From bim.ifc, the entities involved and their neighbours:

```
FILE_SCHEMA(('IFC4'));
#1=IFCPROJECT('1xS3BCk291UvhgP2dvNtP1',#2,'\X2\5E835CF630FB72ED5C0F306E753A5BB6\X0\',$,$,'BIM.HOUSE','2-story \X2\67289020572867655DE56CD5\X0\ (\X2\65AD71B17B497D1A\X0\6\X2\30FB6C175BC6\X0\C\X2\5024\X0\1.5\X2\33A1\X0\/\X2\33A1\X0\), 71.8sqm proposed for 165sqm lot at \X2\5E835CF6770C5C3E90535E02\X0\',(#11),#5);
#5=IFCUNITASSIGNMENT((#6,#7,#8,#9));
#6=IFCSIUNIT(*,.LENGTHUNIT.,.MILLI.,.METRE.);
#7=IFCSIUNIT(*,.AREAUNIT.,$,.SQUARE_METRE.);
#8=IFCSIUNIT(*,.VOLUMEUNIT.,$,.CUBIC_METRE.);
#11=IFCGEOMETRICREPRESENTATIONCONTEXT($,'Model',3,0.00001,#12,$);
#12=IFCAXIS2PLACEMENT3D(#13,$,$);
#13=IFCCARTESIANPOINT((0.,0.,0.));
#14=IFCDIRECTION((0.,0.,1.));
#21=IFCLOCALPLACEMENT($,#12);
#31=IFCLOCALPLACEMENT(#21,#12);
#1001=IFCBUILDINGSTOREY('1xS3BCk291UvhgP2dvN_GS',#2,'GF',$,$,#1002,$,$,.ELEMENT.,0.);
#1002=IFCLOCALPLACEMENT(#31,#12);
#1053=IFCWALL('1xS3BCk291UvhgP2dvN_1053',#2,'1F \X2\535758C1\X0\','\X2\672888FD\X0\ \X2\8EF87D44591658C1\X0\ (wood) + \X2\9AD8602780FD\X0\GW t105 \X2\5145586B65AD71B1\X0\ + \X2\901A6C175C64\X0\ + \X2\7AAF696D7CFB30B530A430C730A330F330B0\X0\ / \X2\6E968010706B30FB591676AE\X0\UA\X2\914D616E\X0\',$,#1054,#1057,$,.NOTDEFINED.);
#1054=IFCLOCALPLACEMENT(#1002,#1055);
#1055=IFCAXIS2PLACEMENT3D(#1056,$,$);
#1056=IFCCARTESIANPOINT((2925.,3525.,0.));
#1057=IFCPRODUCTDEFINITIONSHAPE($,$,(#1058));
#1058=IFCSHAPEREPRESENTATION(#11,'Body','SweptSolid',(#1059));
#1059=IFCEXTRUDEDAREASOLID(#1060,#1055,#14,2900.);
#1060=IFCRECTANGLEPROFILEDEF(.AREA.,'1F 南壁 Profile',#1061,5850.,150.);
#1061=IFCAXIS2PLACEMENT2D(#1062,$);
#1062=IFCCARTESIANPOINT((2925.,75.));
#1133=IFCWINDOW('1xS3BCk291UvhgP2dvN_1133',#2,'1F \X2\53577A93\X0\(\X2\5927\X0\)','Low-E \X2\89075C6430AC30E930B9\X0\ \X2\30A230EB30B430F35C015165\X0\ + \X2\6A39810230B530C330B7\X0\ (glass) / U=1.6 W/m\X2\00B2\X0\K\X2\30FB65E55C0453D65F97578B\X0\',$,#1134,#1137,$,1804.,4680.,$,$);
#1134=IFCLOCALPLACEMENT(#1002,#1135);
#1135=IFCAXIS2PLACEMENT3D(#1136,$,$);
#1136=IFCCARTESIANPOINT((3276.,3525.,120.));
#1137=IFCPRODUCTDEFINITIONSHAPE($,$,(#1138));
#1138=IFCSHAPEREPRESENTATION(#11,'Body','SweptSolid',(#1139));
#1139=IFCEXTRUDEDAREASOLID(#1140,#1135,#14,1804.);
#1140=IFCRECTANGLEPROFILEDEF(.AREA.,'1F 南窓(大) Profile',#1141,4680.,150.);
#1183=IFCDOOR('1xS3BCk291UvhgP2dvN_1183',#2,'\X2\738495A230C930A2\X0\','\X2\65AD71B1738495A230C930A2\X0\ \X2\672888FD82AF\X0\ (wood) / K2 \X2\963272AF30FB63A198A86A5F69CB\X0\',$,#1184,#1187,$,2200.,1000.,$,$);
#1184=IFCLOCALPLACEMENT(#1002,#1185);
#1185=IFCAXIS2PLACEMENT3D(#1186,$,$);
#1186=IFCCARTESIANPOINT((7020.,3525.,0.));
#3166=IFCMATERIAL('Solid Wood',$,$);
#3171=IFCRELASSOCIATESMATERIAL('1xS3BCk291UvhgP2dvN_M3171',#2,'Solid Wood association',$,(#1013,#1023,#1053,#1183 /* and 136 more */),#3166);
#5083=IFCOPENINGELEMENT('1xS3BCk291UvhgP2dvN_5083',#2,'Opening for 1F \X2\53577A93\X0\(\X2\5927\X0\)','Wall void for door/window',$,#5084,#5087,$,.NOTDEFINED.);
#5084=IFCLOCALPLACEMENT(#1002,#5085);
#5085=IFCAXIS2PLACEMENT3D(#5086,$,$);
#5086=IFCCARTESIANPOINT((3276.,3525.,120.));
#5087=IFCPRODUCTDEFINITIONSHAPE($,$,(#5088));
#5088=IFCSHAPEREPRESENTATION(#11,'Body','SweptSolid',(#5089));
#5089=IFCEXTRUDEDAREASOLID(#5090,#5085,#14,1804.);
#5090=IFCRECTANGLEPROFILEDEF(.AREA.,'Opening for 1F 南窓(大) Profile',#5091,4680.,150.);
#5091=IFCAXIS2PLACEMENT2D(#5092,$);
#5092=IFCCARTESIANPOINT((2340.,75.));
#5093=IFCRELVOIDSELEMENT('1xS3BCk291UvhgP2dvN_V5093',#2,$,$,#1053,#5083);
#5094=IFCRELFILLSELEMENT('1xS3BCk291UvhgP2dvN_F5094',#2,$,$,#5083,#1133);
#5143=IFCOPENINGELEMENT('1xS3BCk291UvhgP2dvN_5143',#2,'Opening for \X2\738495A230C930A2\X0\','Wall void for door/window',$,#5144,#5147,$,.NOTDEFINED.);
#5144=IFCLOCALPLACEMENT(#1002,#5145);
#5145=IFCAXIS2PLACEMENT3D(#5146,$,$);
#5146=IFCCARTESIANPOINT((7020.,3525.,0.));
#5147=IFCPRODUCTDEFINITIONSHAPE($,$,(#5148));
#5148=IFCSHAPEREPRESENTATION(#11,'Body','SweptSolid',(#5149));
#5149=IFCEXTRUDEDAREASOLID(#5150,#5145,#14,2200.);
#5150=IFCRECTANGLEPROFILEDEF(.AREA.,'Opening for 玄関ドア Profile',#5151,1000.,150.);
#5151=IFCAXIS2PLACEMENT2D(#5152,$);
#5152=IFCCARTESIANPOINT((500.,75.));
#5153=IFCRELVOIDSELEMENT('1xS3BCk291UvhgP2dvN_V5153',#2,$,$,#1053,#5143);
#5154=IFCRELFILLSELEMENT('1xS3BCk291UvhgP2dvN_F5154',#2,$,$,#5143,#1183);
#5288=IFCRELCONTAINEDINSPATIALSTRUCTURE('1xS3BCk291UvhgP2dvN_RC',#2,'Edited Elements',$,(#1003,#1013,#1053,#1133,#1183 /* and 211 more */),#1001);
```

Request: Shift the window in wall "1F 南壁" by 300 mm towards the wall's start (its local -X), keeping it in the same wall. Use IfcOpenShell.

```python
import ifcopenshell
import ifcopenshell.api.geometry
import ifcopenshell.util.placement
import ifcopenshell.util.unit

model = ifcopenshell.open("bim.ifc")
unit_scale = ifcopenshell.util.unit.calculate_unit_scale(model)

window = model.by_guid("1xS3BCk291UvhgP2dvN_1133")
opening = window.FillsVoids[0].RelatingOpeningElement
wall = opening.VoidsElements[0].RelatingBuildingElement

wall_matrix = ifcopenshell.util.placement.get_local_placement(wall.ObjectPlacement)
shift = wall_matrix[:3, 0] * -0.3 / unit_scale
before = ifcopenshell.util.placement.get_local_placement(window.ObjectPlacement)[:3, 3].copy()

# The window is not placed relative to its opening, so move both.
for product in (opening, window):
    matrix = ifcopenshell.util.placement.get_local_placement(product.ObjectPlacement)
    matrix[:3, 3] += shift
    ifcopenshell.api.geometry.edit_object_placement(model, product=product, matrix=matrix, is_si=False)

after = ifcopenshell.util.placement.get_local_placement(window.ObjectPlacement)[:3, 3]
print("window moved by", (after - before).round(3) + 0.0)

model.write("bim-out.ifc")
```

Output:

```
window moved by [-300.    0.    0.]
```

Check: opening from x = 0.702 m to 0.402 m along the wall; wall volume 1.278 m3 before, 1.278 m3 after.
